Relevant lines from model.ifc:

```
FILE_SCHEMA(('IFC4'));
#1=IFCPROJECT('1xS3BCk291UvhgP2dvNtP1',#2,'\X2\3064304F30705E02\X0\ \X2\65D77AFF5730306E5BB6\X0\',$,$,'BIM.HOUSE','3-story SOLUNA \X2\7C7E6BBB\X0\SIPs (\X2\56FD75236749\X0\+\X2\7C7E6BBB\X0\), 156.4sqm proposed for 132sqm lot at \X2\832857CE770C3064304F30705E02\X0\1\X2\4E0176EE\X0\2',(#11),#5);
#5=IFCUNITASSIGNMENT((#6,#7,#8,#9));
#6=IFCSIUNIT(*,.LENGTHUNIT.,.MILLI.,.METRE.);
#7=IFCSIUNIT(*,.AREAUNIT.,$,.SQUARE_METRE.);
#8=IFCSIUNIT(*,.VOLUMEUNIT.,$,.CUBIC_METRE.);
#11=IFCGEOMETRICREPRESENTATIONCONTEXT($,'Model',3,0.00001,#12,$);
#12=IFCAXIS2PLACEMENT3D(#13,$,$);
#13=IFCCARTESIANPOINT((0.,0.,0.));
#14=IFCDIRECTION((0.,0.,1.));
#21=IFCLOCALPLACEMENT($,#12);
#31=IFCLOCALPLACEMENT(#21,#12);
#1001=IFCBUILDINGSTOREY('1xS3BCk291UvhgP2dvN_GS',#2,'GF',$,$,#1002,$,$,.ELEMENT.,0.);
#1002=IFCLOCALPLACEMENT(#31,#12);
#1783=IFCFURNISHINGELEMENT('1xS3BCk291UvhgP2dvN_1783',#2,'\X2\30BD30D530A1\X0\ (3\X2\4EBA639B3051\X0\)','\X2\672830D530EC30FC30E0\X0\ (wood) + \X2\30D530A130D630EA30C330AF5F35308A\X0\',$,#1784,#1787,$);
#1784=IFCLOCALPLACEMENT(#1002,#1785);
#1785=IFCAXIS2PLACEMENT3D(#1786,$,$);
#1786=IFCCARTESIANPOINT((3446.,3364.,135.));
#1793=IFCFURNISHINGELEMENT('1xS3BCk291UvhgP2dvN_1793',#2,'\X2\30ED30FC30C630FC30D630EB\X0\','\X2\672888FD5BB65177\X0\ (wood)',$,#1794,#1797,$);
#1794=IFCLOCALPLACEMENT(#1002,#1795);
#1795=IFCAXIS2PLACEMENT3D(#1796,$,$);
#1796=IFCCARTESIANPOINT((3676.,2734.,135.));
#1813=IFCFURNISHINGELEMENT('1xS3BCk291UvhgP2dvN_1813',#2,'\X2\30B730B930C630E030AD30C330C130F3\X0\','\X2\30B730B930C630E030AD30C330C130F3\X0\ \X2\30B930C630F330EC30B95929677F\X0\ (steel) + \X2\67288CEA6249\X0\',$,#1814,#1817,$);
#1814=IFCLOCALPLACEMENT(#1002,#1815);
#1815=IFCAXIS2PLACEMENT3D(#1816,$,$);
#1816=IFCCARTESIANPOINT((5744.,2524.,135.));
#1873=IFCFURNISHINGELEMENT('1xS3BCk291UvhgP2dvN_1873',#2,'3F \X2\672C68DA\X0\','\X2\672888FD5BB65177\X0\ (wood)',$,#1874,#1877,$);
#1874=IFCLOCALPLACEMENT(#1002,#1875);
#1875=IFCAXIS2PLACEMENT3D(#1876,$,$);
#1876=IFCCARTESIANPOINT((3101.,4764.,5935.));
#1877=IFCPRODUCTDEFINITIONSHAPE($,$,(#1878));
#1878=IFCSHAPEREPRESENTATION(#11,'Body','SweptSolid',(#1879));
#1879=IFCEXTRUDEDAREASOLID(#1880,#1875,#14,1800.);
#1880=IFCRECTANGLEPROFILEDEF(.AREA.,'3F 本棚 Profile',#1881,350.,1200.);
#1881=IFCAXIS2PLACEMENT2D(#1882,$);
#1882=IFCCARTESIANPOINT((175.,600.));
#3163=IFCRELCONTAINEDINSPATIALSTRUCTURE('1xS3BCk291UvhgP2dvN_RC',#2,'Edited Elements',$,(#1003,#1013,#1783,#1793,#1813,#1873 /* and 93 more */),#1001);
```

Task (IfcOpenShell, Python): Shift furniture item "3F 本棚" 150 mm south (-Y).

```python
import ifcopenshell
import ifcopenshell.api.geometry
import ifcopenshell.util.placement

model = ifcopenshell.open("model.ifc")

item = model.by_guid("1xS3BCk291UvhgP2dvN_1873")
matrix = ifcopenshell.util.placement.get_local_placement(item.ObjectPlacement)
matrix[1, 3] -= 150.0
ifcopenshell.api.geometry.edit_object_placement(model, product=item, matrix=matrix, is_si=False)

print(ifcopenshell.util.placement.get_local_placement(item.ObjectPlacement).round(3) + 0.0)

model.write("model_updated.ifc")
```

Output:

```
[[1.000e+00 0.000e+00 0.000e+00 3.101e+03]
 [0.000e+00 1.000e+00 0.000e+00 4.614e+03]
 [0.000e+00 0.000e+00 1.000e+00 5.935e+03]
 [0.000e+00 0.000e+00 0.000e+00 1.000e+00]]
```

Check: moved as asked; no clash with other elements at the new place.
